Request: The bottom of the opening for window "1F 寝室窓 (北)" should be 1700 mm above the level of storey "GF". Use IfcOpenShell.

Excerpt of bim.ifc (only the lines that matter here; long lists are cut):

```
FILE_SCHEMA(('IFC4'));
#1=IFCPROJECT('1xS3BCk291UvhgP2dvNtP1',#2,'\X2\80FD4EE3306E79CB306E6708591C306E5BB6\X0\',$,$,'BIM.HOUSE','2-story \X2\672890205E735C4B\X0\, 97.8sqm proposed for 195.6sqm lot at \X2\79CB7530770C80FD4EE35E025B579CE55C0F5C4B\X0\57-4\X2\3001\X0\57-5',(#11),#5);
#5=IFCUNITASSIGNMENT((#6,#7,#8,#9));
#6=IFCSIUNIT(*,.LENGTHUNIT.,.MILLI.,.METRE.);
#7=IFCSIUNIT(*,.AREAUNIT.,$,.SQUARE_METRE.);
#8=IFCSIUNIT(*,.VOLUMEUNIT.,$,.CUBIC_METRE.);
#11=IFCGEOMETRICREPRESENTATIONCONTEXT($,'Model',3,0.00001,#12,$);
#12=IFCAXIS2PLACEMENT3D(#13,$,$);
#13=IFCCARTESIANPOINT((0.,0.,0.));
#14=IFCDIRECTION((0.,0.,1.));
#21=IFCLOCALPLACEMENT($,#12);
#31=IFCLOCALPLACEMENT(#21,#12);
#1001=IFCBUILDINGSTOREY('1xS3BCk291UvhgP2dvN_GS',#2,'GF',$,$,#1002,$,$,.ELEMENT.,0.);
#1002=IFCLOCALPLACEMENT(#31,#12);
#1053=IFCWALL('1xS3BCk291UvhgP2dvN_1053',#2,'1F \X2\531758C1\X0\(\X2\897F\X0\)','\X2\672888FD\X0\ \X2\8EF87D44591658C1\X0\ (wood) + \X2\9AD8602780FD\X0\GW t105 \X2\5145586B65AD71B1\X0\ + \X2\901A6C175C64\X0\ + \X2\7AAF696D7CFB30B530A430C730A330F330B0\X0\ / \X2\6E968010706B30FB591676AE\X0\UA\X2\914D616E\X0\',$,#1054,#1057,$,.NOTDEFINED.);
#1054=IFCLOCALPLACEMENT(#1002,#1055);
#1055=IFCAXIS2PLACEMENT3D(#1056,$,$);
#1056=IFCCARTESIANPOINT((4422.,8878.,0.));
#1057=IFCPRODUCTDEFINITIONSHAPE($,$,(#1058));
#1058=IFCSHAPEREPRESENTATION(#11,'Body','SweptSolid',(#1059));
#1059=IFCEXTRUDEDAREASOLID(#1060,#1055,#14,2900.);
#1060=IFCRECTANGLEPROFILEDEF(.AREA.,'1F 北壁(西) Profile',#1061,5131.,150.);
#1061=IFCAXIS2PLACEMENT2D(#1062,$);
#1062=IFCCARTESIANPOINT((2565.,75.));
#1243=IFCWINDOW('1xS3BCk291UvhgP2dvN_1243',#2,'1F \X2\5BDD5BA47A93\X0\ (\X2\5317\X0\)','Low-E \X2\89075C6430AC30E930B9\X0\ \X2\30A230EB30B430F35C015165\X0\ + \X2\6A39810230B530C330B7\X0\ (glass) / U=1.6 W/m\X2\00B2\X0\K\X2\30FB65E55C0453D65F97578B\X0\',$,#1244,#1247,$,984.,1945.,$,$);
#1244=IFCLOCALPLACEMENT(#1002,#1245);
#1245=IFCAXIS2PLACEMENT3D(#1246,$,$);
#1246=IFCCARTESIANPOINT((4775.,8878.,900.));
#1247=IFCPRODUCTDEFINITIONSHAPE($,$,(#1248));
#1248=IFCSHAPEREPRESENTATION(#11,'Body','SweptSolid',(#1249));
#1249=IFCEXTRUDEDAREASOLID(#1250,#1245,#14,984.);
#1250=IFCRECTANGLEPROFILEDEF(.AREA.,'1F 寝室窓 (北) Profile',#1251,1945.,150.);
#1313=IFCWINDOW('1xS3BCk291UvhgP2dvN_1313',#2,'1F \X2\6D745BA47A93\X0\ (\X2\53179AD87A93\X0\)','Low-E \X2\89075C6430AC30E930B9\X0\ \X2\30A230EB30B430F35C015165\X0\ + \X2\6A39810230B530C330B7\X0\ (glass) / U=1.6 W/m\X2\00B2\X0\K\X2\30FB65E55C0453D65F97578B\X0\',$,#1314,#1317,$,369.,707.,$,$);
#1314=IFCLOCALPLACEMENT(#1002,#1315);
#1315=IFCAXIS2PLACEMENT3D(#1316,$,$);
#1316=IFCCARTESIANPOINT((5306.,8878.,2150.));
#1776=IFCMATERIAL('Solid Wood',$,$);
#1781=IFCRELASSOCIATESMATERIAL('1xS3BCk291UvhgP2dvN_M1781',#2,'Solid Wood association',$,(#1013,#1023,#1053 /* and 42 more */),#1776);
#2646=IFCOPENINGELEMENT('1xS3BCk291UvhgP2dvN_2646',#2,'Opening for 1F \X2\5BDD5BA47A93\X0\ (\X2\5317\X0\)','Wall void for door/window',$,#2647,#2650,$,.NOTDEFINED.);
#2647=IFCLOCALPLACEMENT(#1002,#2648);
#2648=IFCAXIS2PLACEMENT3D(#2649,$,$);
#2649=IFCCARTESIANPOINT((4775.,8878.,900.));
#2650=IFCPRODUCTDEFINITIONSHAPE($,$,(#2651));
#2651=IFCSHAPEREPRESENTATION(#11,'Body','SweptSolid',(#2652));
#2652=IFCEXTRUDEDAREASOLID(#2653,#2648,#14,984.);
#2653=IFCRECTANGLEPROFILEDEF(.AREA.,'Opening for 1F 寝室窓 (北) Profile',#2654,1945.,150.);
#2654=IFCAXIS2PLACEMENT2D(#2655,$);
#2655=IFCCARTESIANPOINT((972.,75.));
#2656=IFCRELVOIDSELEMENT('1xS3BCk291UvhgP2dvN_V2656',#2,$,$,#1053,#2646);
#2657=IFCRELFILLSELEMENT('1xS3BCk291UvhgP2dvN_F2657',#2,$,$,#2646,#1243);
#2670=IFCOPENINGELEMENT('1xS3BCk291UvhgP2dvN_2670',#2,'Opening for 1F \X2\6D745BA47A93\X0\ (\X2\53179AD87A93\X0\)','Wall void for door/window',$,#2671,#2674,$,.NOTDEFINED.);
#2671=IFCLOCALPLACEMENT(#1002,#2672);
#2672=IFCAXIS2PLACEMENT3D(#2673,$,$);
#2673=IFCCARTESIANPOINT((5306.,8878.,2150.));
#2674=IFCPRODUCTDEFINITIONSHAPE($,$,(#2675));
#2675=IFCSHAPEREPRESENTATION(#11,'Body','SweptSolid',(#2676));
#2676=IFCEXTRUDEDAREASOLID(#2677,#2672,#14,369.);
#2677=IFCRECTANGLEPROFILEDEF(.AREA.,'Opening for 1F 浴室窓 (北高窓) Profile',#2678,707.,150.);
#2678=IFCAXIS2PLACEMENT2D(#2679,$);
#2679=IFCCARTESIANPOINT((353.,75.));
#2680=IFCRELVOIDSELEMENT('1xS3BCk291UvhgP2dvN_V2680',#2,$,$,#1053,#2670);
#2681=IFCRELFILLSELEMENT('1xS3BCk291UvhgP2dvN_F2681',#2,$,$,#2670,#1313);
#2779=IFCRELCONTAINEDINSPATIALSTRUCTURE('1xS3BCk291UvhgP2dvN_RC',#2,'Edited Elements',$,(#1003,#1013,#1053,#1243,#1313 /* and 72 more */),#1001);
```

```python
import numpy as np
import ifcopenshell
import ifcopenshell.api.geometry
import ifcopenshell.geom
import ifcopenshell.util.element
import ifcopenshell.util.placement
import ifcopenshell.util.shape
import ifcopenshell.util.unit

model = ifcopenshell.open("bim.ifc")
unit_scale = ifcopenshell.util.unit.calculate_unit_scale(model)

window = model.by_guid("1xS3BCk291UvhgP2dvN_1243")
opening = window.FillsVoids[0].RelatingOpeningElement
storey = ifcopenshell.util.element.get_container(window, ifc_class="IfcBuildingStorey")
level = ifcopenshell.util.placement.get_local_placement(storey.ObjectPlacement)[2, 3]

# The opening's origin need not be at the sill, so measure its lowest point.
shape = ifcopenshell.geom.create_shape(ifcopenshell.geom.settings(), opening)
bottom = ifcopenshell.util.shape.get_shape_bottom_elevation(shape, shape.geometry) / unit_scale
dz = level + 1.7 / unit_scale - bottom

shift = np.array([0.0, 0.0, dz])
# The window is not placed relative to its opening, so move both.
for product in (opening, window):
    matrix = ifcopenshell.util.placement.get_local_placement(product.ObjectPlacement)
    matrix[:3, 3] += shift
    ifcopenshell.api.geometry.edit_object_placement(model, product=product, matrix=matrix, is_si=False)

print(f"moved by {dz * unit_scale:+.3f} m")

model.write("bim_v2.ifc")
```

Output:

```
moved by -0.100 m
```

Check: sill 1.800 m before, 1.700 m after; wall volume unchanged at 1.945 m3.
